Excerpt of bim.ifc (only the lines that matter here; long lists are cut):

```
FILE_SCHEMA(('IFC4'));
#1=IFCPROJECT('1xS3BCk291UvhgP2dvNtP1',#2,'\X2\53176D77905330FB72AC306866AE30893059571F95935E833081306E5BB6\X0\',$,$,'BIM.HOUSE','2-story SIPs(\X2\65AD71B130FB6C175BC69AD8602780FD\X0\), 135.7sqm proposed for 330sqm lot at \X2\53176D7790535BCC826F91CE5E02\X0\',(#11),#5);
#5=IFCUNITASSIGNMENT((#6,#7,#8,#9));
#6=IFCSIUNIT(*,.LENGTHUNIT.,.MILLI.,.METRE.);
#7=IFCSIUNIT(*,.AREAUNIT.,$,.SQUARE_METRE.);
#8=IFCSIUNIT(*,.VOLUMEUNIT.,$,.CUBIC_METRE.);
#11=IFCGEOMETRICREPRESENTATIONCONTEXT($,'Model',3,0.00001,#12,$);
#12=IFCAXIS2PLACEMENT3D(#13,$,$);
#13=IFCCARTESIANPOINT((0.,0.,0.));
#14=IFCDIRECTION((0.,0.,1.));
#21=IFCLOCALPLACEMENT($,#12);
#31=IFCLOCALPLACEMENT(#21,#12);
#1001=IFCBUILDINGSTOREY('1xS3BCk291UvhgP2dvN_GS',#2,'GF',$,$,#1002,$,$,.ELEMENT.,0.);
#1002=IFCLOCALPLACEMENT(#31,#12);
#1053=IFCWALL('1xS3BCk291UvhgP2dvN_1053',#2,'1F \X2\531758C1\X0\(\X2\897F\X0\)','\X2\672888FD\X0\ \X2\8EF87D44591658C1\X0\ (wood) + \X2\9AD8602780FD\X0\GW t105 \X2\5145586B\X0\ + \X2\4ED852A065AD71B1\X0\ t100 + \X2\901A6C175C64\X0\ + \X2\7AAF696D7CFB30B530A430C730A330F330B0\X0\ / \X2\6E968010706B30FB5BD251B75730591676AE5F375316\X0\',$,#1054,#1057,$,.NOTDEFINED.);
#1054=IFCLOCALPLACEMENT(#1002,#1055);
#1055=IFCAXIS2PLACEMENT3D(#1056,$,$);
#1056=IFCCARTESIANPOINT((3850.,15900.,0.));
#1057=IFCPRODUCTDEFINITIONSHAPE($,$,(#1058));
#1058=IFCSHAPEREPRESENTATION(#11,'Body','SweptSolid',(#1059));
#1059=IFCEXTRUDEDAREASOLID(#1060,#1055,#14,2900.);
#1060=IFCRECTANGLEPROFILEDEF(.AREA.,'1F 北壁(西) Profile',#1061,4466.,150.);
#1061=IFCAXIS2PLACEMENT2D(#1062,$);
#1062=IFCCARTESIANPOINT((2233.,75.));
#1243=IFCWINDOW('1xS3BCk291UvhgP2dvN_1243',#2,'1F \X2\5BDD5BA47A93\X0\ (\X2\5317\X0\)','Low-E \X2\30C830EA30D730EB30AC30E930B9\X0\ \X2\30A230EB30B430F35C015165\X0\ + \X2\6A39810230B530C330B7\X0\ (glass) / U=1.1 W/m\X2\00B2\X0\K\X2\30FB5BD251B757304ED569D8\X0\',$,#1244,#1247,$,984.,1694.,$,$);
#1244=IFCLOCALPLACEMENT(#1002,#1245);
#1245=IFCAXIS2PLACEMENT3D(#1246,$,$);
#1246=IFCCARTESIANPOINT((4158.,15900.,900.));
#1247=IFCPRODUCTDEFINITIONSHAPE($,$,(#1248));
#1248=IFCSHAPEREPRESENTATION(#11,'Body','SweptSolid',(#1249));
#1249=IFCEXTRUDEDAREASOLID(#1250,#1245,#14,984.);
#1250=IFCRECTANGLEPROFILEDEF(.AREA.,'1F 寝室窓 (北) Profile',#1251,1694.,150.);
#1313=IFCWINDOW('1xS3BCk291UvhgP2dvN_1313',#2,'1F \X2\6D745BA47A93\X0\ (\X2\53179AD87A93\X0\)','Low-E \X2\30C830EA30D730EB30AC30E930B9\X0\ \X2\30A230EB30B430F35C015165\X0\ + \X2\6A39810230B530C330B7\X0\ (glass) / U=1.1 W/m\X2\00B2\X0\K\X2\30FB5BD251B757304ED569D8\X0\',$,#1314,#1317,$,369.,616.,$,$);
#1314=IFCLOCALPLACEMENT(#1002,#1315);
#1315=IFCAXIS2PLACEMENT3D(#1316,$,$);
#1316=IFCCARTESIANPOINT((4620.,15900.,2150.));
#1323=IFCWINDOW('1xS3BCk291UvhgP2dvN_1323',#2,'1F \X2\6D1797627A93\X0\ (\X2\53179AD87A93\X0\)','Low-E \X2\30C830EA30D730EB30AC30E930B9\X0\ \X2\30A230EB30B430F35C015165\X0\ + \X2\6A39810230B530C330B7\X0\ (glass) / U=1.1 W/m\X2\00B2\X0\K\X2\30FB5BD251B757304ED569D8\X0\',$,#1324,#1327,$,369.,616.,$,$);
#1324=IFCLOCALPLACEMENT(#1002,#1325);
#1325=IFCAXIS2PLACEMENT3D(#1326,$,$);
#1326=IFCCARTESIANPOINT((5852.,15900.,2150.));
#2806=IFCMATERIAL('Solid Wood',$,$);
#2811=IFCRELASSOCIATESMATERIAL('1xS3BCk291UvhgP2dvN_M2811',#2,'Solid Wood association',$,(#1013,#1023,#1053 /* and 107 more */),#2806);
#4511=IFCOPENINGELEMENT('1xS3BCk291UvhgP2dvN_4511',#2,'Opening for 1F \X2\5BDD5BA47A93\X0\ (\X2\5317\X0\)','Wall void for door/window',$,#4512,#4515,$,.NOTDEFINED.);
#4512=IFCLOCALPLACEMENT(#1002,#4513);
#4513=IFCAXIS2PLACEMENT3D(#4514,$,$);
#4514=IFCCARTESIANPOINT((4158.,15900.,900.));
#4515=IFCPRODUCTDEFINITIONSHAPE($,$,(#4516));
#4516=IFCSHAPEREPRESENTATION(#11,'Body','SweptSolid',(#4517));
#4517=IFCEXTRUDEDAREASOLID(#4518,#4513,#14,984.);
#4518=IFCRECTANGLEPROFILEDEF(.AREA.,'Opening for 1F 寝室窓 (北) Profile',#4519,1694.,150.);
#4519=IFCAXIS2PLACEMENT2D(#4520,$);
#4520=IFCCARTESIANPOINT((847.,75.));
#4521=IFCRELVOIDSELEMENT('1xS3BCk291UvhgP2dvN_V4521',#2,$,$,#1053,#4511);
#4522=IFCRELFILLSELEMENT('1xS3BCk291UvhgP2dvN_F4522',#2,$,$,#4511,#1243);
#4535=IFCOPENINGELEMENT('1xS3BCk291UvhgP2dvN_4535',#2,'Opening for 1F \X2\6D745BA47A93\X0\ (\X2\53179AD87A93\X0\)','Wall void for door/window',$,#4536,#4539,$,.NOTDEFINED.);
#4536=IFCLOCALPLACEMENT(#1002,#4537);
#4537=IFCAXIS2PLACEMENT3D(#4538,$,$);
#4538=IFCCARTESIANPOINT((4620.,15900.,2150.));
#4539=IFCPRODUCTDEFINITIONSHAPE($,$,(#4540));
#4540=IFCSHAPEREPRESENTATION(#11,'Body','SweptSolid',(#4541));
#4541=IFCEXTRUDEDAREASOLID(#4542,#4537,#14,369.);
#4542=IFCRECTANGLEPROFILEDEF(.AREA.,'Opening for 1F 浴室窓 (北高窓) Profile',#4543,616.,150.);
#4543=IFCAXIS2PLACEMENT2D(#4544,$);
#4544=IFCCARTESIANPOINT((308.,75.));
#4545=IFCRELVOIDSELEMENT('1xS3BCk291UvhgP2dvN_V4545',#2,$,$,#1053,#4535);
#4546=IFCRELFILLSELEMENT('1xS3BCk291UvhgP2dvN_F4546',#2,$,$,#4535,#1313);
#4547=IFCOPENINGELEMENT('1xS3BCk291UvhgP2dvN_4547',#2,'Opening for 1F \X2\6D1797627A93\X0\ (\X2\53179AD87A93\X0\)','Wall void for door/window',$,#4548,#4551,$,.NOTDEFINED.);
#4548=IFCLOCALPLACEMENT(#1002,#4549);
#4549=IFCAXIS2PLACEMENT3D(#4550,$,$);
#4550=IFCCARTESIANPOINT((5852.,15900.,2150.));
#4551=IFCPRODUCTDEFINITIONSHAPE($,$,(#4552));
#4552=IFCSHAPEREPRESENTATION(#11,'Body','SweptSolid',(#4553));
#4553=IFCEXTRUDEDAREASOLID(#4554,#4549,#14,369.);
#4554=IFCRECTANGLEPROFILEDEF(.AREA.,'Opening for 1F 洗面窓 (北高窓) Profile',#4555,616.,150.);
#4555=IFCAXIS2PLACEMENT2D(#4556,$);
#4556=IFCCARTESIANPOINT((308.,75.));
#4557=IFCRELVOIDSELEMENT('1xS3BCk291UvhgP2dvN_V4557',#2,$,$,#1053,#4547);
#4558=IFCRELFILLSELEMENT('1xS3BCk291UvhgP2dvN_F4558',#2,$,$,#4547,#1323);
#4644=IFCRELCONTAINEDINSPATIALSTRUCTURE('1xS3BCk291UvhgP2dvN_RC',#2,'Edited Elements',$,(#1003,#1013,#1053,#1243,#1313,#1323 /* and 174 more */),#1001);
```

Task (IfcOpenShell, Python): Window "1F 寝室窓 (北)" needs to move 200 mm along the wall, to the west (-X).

```python
import ifcopenshell
import ifcopenshell.api.geometry
import ifcopenshell.util.placement
import ifcopenshell.util.unit

model = ifcopenshell.open("bim.ifc")
unit_scale = ifcopenshell.util.unit.calculate_unit_scale(model)

window = model.by_id(1243)
opening = window.FillsVoids[0].RelatingOpeningElement
wall = opening.VoidsElements[0].RelatingBuildingElement

wall_matrix = ifcopenshell.util.placement.get_local_placement(wall.ObjectPlacement)
shift = wall_matrix[:3, 0] * -0.2 / unit_scale
before = ifcopenshell.util.placement.get_local_placement(window.ObjectPlacement)[:3, 3].copy()

# The window is not placed relative to its opening, so move both.
for product in (opening, window):
    matrix = ifcopenshell.util.placement.get_local_placement(product.ObjectPlacement)
    matrix[:3, 3] += shift
    ifcopenshell.api.geometry.edit_object_placement(model, product=product, matrix=matrix, is_si=False)

after = ifcopenshell.util.placement.get_local_placement(window.ObjectPlacement)[:3, 3]
print("window moved by", (after - before).round(3) + 0.0)

model.write("bim_edited.ifc")
```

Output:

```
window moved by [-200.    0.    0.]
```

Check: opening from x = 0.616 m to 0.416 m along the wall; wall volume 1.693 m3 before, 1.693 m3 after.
